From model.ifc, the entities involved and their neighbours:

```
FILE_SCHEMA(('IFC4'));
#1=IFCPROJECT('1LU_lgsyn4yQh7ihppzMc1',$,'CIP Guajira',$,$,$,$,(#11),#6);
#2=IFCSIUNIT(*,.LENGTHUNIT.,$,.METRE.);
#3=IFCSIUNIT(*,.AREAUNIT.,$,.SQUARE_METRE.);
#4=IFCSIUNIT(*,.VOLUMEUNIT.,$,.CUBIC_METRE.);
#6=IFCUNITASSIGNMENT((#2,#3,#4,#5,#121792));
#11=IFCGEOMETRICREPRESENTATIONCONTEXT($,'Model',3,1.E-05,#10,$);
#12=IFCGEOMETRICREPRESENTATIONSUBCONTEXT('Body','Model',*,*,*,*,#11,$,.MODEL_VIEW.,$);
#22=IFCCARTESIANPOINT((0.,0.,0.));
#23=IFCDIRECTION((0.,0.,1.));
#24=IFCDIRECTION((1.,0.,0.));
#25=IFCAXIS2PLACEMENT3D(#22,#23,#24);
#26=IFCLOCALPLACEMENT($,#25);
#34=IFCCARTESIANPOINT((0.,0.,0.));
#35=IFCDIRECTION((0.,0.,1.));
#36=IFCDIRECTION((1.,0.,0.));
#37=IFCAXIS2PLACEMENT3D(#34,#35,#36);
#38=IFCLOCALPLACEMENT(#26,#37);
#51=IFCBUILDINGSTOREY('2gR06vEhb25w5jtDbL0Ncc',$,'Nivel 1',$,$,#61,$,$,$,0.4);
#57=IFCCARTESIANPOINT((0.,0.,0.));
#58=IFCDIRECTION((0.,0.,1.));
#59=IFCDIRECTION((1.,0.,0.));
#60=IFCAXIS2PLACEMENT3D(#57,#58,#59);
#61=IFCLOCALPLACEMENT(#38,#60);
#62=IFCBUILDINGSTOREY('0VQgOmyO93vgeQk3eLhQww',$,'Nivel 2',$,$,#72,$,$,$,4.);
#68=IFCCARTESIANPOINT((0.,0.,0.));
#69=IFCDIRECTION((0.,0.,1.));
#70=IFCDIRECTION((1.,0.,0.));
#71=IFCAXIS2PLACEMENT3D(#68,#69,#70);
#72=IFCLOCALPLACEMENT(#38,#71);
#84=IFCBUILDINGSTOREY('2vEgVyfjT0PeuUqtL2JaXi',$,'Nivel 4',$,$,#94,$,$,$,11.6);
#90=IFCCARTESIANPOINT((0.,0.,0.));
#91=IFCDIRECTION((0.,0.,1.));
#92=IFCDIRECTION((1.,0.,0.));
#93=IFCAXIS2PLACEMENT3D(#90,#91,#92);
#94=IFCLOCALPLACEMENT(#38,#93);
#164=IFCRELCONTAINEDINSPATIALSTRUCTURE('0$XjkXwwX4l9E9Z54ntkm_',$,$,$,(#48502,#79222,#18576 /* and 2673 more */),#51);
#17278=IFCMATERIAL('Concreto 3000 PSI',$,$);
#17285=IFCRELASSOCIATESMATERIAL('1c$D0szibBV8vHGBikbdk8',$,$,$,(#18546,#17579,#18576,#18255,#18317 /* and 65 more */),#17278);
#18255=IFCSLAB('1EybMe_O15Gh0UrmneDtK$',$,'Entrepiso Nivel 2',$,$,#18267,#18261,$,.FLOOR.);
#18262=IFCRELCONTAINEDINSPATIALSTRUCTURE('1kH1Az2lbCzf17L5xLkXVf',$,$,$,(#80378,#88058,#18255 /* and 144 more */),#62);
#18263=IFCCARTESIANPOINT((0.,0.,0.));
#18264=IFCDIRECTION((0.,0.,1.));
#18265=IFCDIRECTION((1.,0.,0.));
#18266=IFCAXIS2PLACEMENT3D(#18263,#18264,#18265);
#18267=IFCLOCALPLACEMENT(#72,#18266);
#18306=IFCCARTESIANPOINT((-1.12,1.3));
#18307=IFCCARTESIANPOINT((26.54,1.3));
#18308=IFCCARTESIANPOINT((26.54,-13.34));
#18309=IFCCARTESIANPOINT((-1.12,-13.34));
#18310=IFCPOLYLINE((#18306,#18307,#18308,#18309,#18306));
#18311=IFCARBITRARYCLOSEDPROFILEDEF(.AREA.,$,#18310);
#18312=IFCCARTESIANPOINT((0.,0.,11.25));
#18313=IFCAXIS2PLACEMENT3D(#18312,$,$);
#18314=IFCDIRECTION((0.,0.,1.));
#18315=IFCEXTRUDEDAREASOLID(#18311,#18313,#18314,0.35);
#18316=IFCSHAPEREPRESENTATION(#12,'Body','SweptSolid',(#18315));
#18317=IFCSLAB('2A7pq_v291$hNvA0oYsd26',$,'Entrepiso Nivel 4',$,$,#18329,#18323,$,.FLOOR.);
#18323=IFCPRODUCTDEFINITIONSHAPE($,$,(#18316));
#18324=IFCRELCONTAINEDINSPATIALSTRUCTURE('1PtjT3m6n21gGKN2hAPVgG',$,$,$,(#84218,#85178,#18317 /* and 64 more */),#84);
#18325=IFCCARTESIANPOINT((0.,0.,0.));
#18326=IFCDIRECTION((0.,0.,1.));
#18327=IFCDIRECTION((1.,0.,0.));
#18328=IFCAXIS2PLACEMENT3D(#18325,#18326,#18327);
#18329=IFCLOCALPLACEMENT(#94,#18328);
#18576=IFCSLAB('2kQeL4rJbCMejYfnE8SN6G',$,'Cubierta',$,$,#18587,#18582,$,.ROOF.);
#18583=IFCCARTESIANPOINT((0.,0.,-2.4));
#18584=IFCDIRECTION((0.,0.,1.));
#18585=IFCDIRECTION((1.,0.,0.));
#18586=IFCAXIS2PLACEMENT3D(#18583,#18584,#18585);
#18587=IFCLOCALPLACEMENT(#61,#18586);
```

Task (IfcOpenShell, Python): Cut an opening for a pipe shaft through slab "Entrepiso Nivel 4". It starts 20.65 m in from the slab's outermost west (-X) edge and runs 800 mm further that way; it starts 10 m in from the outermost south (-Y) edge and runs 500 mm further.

```python
import numpy as np
import ifcopenshell
import ifcopenshell.api.feature
import ifcopenshell.api.geometry
import ifcopenshell.api.root
import ifcopenshell.geom
import ifcopenshell.util.placement
import ifcopenshell.util.representation
import ifcopenshell.util.shape
import ifcopenshell.util.unit

model = ifcopenshell.open("model.ifc")
unit_scale = ifcopenshell.util.unit.calculate_unit_scale(model)
settings = ifcopenshell.geom.settings()


def volume(element):
    """Net volume in cubic metres, openings subtracted."""
    shape = ifcopenshell.geom.create_shape(settings, element)
    return ifcopenshell.util.shape.get_volume(shape.geometry)


slab = model.by_guid("2A7pq_v291$hNvA0oYsd26")
before = volume(slab)

# Extent in the slab's own axes, in metres. The edges named are its -X and -Y sides.
slab_shape = ifcopenshell.geom.create_shape(settings, slab)
vertices = ifcopenshell.util.shape.get_vertices(slab_shape.geometry)
x_min, y_min, bottom = vertices.min(axis=0)
top = vertices[:, 2].max()

opening = ifcopenshell.api.root.create_entity(model, ifc_class="IfcOpeningElement", name="Pipe shaft opening", predefined_type="OPENING")
context = ifcopenshell.util.representation.get_context(model, "Model", "Body", "MODEL_VIEW")
width, depth = 0.8, 0.5
outline = [(0.0, 0.0), (width, 0.0), (width, depth), (0.0, depth), (0.0, 0.0)]
# Overshoot both faces by 50 mm so the cut is clean.
shape = ifcopenshell.api.geometry.add_slab_representation(
    model, context=context, depth=top - bottom + 0.1, polyline=outline
)
ifcopenshell.api.geometry.assign_representation(model, product=opening, representation=shape)

matrix = ifcopenshell.util.placement.get_local_placement(slab.ObjectPlacement)
matrix[:, 3] = matrix @ np.append(np.array([x_min + 20.65, y_min + 10, bottom - 0.05]) / unit_scale, 1.0)
ifcopenshell.api.geometry.edit_object_placement(model, product=opening, matrix=matrix, is_si=False)
ifcopenshell.api.feature.add_feature(model, feature=opening, element=slab)

after = volume(slab)

print(f"slab volume {before:.3f} -> {after:.3f} m3")

model.write("model_v2.ifc")
```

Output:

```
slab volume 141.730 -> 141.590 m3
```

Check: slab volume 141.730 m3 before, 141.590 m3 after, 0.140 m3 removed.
